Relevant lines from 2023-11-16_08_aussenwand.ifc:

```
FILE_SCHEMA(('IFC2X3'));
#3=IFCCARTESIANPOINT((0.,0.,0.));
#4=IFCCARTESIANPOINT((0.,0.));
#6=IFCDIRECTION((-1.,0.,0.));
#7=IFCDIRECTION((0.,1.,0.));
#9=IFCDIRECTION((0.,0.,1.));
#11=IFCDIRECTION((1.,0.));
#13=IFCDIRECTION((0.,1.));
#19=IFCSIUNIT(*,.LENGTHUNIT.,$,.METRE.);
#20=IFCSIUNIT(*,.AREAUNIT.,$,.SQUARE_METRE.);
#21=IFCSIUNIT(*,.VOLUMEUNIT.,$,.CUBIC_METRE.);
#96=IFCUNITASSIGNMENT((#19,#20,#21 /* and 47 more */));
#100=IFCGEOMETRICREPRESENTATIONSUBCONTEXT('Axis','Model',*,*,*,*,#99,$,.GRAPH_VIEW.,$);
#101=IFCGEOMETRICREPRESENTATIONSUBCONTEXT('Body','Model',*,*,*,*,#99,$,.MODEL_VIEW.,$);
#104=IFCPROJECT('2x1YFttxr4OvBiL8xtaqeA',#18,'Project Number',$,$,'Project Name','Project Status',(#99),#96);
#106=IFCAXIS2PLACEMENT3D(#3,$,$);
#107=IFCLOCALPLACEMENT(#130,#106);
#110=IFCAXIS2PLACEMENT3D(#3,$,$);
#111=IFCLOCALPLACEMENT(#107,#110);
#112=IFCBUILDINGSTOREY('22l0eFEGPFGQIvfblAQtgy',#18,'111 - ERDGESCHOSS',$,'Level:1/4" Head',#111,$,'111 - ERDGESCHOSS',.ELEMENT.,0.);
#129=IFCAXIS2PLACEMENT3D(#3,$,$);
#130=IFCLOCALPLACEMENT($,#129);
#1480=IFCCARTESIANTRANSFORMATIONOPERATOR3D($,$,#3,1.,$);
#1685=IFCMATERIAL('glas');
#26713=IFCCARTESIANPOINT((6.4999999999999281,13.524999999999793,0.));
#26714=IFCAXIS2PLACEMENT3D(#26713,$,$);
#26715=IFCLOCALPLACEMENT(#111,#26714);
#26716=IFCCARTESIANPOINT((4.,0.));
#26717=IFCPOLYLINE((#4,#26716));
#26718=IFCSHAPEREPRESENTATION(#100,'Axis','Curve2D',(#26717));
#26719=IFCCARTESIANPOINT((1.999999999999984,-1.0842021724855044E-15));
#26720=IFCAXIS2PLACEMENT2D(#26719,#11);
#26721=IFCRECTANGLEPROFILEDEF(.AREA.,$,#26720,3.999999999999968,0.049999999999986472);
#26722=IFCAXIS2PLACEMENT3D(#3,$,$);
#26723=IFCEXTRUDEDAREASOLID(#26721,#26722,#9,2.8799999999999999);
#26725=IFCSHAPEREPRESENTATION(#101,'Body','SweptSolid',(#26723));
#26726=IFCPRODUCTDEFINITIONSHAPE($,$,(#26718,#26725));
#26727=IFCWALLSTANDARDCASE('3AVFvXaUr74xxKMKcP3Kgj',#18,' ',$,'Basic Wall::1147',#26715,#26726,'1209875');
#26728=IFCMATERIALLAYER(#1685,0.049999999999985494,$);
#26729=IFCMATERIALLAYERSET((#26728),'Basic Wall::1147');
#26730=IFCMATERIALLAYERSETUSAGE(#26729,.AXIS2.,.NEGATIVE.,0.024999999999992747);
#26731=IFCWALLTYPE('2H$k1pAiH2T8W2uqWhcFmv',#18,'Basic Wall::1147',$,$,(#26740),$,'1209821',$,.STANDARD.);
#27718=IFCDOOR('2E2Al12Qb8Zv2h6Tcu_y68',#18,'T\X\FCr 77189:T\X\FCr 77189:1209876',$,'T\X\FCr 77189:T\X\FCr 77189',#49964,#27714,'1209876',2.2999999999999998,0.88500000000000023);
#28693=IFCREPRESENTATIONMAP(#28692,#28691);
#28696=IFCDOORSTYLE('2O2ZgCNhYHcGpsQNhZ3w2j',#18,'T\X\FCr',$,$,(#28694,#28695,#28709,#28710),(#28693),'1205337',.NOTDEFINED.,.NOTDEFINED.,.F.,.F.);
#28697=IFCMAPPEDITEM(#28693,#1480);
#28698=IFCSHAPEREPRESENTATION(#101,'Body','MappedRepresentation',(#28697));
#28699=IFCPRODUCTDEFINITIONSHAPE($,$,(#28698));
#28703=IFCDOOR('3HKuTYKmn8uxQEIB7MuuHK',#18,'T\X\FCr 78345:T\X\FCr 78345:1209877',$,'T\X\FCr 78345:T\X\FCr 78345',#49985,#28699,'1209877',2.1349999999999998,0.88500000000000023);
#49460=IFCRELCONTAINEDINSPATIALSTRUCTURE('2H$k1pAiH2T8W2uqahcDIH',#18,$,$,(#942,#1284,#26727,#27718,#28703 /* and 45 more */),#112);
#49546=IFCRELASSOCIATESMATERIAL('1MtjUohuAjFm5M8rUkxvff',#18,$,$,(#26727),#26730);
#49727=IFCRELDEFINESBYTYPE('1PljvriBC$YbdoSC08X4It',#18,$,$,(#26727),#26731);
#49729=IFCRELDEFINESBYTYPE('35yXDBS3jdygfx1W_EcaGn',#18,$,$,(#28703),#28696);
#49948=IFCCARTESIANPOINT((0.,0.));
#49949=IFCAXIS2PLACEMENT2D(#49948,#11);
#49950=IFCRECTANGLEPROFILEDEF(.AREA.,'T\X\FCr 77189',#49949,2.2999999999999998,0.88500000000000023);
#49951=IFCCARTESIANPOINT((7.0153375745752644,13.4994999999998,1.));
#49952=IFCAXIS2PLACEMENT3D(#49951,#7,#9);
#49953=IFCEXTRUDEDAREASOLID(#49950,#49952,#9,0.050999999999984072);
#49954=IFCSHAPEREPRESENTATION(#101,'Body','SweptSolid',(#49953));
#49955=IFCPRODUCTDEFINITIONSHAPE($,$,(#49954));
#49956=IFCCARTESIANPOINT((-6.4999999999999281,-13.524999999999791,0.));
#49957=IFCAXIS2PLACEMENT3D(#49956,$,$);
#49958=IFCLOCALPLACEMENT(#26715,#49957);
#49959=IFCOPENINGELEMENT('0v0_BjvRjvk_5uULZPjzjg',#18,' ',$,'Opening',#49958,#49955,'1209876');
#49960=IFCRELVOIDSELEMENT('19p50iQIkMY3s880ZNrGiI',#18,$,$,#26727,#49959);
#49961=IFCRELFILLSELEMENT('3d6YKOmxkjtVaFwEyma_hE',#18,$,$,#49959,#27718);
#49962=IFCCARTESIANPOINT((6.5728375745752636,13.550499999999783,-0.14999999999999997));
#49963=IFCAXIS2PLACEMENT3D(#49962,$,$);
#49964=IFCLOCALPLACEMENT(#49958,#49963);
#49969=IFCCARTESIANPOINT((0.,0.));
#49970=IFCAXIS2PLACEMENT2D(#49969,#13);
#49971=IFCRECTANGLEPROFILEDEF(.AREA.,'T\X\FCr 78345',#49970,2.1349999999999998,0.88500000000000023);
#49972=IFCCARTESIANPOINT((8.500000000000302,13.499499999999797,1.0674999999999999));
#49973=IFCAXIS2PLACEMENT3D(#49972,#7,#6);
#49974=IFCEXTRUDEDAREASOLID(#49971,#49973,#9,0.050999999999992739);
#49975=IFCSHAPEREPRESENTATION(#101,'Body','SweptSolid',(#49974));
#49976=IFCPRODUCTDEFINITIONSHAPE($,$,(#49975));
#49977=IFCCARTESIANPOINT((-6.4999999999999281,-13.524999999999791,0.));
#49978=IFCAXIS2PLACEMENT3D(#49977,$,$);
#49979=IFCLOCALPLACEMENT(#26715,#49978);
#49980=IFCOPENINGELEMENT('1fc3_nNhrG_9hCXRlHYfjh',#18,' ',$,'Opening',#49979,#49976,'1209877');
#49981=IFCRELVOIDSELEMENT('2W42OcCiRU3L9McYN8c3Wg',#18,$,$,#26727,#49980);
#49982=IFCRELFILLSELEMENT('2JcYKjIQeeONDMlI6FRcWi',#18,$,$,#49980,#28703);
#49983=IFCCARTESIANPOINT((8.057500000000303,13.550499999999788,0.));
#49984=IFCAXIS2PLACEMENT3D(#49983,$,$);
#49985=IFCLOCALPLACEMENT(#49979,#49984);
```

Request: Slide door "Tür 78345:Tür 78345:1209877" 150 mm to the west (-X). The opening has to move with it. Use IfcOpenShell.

```python
import ifcopenshell
import ifcopenshell.api.geometry
import ifcopenshell.util.placement
import ifcopenshell.util.unit

model = ifcopenshell.open("2023-11-16_08_aussenwand.ifc")
unit_scale = ifcopenshell.util.unit.calculate_unit_scale(model)

door = model.by_guid("3HKuTYKmn8uxQEIB7MuuHK")
opening = door.FillsVoids[0].RelatingOpeningElement
wall = opening.VoidsElements[0].RelatingBuildingElement

wall_matrix = ifcopenshell.util.placement.get_local_placement(wall.ObjectPlacement)
shift = wall_matrix[:3, 0] * -0.15 / unit_scale
before = ifcopenshell.util.placement.get_local_placement(door.ObjectPlacement)[:3, 3].copy()

# The door is placed relative to its opening, so it follows when the opening moves.
matrix = ifcopenshell.util.placement.get_local_placement(opening.ObjectPlacement)
matrix[:3, 3] += shift
ifcopenshell.api.geometry.edit_object_placement(
    model, product=opening, matrix=matrix, is_si=False, should_transform_children=True
)

after = ifcopenshell.util.placement.get_local_placement(door.ObjectPlacement)[:3, 3]
print("door moved by", (after - before).round(3) + 0.0)

model.write("2023-11-16_08_aussenwand_v2.ifc")
```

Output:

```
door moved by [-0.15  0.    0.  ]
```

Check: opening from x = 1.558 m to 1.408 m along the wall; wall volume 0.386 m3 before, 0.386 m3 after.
